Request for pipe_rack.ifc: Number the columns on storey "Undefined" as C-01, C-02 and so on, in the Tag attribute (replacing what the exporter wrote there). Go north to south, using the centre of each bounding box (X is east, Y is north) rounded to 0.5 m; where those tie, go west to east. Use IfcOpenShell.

First a look at what the model holds.

```python
import ifcopenshell
import ifcopenshell.util.element
import ifcopenshell.util.placement

model = ifcopenshell.open("pipe_rack.ifc")
print(model.schema)
storey = next(s for s in model.by_type("IfcBuildingStorey") if s.Name == "Undefined")
columns = [e for e in ifcopenshell.util.element.get_decomposition(storey) if e.is_a("IfcColumn")]
for e in sorted(columns, key=lambda e: e.id()):
    origin = ifcopenshell.util.placement.get_local_placement(e.ObjectPlacement)[:3, 3]
    print(e.id(), e.Tag, e.Name, origin.round(2) + 0.0, sep=" | ")
```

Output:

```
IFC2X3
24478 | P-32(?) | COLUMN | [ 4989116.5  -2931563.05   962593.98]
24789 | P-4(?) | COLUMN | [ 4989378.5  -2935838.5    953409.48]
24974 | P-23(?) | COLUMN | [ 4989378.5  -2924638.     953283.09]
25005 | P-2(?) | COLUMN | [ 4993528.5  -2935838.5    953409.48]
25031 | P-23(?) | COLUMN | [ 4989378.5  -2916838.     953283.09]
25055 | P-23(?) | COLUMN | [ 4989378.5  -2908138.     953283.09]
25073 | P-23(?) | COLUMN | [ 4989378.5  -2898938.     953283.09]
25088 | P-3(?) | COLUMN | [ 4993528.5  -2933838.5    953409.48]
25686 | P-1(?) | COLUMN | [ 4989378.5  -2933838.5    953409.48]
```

```python
import ifcopenshell
import ifcopenshell.geom
import ifcopenshell.util.element
import ifcopenshell.util.shape

model = ifcopenshell.open("pipe_rack.ifc")
settings = ifcopenshell.geom.settings()
settings.set("use-world-coords", True)


def centre(element):
    shape = ifcopenshell.geom.create_shape(settings, element)
    return ifcopenshell.util.shape.get_bbox_centroid(shape.geometry)


storey = next(s for s in model.by_type("IfcBuildingStorey") if s.Name == "Undefined")
columns = [e for e in ifcopenshell.util.element.get_decomposition(storey) if e.is_a("IfcColumn")]

# Insertion points can sit at a corner or the storey origin, so sort by the geometry (in metres).
centres = {e: centre(e) for e in columns}
columns.sort(key=lambda e: (-round(centres[e][1] / 0.5), centres[e][0]))

for i, e in enumerate(columns, start=1):
    number = f"C-{i:02d}"
    e.Tag = number
    print(e.id(), number)

model.write("pipe_rack_edited.ifc")
```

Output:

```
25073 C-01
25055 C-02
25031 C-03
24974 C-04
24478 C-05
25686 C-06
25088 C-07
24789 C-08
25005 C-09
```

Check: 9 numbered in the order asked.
